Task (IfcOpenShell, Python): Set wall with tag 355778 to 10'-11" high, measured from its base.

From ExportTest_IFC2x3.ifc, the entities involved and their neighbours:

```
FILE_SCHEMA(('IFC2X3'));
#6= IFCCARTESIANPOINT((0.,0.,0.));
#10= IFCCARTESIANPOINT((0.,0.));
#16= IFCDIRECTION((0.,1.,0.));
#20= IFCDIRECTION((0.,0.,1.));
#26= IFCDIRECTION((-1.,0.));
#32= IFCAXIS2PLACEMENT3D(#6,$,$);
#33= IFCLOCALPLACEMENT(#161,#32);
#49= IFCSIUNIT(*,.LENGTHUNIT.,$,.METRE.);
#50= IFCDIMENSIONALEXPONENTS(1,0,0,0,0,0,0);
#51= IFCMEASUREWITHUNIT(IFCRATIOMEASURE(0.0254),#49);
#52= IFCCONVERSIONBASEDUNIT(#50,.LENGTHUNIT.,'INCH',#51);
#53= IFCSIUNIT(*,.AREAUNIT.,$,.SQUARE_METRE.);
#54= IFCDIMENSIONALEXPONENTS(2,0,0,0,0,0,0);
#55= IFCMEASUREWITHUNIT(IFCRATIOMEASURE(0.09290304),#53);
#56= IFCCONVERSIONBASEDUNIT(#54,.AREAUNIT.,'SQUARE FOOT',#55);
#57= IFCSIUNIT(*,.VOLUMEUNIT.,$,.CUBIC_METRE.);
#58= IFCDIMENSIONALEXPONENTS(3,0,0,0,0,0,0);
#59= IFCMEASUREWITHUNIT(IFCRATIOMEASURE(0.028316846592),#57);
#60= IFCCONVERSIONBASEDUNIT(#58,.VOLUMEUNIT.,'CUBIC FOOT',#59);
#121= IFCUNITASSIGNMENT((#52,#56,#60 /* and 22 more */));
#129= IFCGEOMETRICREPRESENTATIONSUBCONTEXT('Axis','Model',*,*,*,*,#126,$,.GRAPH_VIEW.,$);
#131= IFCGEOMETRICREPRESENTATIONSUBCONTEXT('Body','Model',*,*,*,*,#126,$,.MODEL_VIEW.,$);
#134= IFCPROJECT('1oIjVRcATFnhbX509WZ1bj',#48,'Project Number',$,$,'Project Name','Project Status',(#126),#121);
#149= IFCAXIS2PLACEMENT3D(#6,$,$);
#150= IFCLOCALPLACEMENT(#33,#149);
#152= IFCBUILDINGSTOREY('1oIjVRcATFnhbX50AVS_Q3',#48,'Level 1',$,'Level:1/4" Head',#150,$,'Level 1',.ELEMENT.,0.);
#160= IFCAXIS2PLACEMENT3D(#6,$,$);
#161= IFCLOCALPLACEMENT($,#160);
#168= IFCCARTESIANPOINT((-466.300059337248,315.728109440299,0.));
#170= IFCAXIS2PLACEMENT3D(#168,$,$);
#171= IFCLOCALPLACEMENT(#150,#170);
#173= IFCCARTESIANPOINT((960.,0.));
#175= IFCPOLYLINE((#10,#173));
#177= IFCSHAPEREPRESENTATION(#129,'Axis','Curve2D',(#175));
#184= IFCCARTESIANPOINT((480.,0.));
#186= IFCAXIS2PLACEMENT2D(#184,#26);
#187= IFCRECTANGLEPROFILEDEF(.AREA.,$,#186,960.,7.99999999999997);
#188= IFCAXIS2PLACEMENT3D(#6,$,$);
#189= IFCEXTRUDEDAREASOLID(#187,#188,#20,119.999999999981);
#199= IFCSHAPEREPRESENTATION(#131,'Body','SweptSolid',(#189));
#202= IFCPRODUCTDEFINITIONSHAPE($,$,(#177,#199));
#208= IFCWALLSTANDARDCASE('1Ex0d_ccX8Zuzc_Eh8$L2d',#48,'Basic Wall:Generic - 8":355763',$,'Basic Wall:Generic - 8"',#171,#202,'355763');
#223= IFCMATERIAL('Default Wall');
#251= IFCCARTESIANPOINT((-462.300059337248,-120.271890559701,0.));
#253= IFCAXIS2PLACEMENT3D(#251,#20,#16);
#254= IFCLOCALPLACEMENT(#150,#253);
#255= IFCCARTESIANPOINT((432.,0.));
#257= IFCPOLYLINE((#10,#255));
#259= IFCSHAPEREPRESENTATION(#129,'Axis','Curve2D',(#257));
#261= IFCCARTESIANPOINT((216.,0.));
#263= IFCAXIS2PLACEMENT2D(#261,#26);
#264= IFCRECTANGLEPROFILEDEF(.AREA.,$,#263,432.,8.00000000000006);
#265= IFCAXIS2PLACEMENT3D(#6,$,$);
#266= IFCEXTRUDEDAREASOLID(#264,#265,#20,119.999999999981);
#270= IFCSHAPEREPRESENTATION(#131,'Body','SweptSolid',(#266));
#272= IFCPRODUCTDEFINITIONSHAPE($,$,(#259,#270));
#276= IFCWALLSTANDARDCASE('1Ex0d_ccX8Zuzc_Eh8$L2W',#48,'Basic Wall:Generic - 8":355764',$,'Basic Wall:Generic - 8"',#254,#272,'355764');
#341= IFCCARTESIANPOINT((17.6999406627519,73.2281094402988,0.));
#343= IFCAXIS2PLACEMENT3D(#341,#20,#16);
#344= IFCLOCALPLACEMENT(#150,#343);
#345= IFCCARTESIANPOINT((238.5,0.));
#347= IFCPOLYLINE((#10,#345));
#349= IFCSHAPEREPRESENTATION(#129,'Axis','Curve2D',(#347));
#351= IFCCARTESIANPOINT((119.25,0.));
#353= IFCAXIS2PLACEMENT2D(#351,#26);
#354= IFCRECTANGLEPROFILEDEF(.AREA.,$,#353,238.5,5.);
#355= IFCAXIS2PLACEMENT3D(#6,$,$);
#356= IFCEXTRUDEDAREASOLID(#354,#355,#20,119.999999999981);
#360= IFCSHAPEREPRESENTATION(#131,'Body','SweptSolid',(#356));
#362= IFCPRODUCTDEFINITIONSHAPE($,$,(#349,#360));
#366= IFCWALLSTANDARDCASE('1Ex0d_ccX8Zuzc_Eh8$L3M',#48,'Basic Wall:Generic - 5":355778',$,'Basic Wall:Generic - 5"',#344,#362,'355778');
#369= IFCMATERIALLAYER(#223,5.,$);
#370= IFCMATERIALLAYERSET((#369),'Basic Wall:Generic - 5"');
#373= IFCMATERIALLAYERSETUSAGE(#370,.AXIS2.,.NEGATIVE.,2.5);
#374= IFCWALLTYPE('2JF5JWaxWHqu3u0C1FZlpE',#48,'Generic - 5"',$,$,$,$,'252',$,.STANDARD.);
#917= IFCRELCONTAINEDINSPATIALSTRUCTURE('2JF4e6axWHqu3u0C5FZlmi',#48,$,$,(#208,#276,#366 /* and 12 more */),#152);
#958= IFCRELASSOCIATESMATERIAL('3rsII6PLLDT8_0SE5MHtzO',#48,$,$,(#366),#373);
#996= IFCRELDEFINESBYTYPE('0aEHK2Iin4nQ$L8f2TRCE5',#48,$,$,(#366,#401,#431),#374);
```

```python
import ifcopenshell
import ifcopenshell.geom
import ifcopenshell.util.representation
import ifcopenshell.util.shape
import ifcopenshell.util.unit

model = ifcopenshell.open("ExportTest_IFC2x3.ifc")
unit_scale = ifcopenshell.util.unit.calculate_unit_scale(model)
settings = ifcopenshell.geom.settings()


def volume(element):
    """Net volume in cubic metres, openings subtracted."""
    shape = ifcopenshell.geom.create_shape(settings, element)
    return ifcopenshell.util.shape.get_volume(shape.geometry)


wall = model.by_guid("1Ex0d_ccX8Zuzc_Eh8$L3M")
before = volume(wall)

body = ifcopenshell.util.representation.get_representation(wall, "Model", "Body")
solid = body.Items[0]
old_height = solid.Depth
solid.Depth = 131 * 0.0254 / unit_scale
after = volume(wall)

print(f"height {old_height:g} -> {solid.Depth:g}, volume {before:.3f} -> {after:.3f} m3")

model.write("ExportTest_IFC2x3_rev.ifc")
```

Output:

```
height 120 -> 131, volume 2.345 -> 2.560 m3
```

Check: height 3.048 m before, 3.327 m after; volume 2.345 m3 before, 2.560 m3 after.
